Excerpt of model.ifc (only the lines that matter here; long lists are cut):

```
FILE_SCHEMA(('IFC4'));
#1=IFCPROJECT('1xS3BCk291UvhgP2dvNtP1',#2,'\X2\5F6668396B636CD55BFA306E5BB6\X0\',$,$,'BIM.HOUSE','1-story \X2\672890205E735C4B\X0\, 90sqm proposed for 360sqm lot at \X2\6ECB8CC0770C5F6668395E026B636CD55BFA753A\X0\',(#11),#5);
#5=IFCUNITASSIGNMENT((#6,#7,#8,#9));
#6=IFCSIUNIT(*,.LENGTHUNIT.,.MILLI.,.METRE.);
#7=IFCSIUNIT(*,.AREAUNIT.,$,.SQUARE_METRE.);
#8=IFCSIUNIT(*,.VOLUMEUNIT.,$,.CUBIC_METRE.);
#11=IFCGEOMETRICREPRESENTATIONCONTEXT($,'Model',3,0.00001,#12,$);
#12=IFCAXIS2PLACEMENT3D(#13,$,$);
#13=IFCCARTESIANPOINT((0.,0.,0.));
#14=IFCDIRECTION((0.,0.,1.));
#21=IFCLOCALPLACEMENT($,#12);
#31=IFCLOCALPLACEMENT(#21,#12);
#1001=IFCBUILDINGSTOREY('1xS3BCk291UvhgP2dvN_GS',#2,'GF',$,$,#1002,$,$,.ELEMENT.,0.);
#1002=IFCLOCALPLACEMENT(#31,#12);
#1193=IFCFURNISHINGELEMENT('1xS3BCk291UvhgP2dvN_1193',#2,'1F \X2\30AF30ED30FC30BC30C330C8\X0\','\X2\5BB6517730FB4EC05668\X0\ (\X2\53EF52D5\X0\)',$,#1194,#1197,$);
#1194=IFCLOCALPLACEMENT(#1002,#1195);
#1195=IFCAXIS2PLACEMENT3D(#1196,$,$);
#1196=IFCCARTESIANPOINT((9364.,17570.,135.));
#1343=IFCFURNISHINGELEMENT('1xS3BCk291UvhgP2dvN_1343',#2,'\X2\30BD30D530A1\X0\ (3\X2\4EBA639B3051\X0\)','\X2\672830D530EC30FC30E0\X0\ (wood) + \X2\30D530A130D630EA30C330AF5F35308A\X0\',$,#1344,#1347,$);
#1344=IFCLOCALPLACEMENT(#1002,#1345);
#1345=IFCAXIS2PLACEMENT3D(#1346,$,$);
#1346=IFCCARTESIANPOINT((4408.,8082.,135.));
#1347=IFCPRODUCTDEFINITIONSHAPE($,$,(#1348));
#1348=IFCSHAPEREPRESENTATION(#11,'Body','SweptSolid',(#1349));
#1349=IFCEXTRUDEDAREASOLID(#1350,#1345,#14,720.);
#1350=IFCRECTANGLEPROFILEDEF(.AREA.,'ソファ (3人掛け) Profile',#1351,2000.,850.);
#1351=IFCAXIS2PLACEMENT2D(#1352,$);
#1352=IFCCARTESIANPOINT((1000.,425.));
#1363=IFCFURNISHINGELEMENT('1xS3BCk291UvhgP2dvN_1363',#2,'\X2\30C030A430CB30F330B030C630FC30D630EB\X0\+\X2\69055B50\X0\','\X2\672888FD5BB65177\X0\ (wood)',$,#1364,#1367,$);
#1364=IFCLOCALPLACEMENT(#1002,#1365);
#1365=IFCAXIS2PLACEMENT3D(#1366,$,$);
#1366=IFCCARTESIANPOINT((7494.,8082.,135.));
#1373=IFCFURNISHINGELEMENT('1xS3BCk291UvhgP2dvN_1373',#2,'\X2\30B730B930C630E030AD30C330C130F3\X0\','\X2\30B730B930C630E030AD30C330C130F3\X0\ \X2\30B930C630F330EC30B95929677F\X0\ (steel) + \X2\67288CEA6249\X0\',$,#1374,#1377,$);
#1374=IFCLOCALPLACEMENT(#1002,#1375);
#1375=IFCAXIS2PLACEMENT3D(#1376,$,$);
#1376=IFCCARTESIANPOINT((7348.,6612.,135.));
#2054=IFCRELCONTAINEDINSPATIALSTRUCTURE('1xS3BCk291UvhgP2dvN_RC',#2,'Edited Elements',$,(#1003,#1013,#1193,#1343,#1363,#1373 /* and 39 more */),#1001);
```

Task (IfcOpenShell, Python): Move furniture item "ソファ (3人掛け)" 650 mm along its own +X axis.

```python
import ifcopenshell
import ifcopenshell.api.geometry
import ifcopenshell.util.placement
import ifcopenshell.util.unit

model = ifcopenshell.open("model.ifc")
unit_scale = ifcopenshell.util.unit.calculate_unit_scale(model)

item = model.by_guid("1xS3BCk291UvhgP2dvN_1343")
matrix = ifcopenshell.util.placement.get_local_placement(item.ObjectPlacement)
matrix[:3, 3] += matrix[:3, 0] * 0.65 / unit_scale
ifcopenshell.api.geometry.edit_object_placement(model, product=item, matrix=matrix, is_si=False)

print(ifcopenshell.util.placement.get_local_placement(item.ObjectPlacement).round(3) + 0.0)

model.write("model-out.ifc")
```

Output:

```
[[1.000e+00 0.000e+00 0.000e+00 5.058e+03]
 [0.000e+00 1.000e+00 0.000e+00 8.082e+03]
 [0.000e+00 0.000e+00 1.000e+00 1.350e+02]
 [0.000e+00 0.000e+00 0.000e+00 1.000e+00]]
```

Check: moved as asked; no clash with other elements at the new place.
